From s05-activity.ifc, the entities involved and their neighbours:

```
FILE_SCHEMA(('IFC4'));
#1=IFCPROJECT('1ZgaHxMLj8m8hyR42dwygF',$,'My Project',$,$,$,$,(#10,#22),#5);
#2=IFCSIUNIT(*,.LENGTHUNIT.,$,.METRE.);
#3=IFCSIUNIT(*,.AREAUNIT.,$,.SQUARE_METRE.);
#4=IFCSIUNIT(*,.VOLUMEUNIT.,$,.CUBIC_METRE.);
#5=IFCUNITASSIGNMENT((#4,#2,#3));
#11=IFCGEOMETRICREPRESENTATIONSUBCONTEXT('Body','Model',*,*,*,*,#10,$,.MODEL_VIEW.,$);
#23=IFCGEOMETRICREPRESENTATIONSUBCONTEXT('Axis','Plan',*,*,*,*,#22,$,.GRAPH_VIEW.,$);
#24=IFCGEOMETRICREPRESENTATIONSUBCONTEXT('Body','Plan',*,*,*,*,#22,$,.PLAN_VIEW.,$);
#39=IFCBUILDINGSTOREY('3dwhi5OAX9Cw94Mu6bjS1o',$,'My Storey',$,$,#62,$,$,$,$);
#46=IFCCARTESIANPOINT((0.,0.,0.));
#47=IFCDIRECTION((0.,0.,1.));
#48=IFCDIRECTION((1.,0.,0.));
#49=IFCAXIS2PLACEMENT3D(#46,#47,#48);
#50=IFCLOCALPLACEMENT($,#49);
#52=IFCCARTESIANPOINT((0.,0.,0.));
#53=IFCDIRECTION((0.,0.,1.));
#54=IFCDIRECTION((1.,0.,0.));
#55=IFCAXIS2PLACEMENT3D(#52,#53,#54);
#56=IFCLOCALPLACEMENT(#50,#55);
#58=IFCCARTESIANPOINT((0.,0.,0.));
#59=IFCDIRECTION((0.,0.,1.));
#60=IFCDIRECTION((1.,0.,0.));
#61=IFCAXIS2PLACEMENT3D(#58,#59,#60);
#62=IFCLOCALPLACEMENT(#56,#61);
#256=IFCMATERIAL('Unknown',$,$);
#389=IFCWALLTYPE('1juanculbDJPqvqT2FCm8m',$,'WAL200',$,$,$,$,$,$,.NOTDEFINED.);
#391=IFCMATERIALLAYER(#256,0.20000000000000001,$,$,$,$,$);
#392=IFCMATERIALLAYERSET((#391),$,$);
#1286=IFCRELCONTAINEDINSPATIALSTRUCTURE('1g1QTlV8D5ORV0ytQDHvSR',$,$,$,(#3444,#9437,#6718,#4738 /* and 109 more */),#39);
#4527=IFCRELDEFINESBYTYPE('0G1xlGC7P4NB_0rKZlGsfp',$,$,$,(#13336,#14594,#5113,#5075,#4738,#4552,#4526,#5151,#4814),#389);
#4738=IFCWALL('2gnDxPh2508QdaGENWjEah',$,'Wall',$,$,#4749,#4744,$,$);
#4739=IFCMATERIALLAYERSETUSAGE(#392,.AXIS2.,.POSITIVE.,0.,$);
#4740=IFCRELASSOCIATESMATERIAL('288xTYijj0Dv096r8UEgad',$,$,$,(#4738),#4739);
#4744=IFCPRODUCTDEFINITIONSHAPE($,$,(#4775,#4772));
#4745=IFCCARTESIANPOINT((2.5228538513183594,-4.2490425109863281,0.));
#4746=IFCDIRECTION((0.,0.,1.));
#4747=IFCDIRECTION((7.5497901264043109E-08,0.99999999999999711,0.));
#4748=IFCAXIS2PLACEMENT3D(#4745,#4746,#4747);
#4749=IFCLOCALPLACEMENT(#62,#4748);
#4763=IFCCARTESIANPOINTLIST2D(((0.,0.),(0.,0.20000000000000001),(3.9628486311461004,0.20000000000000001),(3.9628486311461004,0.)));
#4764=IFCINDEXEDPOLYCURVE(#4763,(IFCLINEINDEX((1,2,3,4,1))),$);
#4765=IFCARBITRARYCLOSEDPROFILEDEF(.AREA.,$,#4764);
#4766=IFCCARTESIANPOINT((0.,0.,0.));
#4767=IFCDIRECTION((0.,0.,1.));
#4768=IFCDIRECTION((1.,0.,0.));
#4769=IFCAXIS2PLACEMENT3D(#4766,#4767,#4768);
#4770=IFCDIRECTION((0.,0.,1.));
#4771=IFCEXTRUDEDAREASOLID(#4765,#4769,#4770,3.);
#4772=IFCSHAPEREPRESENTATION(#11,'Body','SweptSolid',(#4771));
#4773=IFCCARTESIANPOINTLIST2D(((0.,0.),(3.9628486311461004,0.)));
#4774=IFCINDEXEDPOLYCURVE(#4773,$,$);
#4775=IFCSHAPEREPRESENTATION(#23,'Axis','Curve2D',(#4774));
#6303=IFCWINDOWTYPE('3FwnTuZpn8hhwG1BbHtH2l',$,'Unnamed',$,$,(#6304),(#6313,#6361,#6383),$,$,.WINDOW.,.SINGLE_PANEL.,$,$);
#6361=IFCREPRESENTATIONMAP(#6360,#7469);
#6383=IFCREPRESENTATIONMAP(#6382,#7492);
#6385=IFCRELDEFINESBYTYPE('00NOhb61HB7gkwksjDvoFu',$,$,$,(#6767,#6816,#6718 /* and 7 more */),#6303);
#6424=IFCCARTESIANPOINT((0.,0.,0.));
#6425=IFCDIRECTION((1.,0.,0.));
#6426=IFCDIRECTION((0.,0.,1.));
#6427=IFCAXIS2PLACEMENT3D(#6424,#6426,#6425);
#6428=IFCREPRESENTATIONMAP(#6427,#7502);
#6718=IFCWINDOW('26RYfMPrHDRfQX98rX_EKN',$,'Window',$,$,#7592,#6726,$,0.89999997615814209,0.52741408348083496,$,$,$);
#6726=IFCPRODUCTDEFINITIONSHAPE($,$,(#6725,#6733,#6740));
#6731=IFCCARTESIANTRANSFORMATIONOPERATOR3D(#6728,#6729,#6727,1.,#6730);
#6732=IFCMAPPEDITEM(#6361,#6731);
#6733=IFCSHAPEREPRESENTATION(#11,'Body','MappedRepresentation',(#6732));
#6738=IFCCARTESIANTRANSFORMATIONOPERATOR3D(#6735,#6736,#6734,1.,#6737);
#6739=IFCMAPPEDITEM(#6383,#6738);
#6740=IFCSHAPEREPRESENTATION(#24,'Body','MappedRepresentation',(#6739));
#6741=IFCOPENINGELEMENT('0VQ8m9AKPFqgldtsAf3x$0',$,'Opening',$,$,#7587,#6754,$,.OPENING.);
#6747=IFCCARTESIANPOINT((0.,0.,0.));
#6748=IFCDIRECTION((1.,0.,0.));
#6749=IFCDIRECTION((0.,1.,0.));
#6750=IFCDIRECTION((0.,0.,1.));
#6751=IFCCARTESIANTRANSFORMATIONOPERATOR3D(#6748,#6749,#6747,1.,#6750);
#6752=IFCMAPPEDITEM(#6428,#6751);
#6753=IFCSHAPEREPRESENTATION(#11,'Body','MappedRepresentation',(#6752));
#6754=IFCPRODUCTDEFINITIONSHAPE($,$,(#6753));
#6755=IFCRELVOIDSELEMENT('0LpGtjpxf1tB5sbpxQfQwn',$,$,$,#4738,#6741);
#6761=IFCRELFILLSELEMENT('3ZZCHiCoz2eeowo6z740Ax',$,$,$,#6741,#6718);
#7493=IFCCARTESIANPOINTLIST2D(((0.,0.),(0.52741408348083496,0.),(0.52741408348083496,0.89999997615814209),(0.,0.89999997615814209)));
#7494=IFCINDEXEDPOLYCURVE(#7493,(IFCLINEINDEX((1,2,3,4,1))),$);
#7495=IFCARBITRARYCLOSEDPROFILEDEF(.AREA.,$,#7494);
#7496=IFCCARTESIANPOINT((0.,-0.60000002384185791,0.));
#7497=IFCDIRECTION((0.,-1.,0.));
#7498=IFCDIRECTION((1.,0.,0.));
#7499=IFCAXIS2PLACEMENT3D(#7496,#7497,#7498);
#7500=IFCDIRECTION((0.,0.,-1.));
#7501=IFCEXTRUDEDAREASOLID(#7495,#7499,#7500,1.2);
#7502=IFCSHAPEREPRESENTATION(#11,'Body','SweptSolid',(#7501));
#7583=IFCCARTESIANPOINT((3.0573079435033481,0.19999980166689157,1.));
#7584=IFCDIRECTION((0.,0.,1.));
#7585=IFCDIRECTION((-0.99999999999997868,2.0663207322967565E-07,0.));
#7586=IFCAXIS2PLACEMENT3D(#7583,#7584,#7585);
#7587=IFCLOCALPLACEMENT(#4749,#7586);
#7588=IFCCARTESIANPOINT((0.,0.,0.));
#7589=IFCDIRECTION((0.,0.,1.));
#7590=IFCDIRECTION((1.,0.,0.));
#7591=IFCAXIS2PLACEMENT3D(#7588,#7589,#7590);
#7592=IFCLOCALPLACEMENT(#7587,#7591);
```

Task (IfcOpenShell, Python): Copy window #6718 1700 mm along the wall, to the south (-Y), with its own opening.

```python
import ifcopenshell
import ifcopenshell.api.feature
import ifcopenshell.api.geometry
import ifcopenshell.api.root
import ifcopenshell.geom
import ifcopenshell.util.element
import ifcopenshell.util.placement
import ifcopenshell.util.shape
import ifcopenshell.util.unit

model = ifcopenshell.open("s05-activity.ifc")
unit_scale = ifcopenshell.util.unit.calculate_unit_scale(model)
settings = ifcopenshell.geom.settings()


def volume(element):
    """Net volume in cubic metres, openings subtracted."""
    shape = ifcopenshell.geom.create_shape(settings, element)
    return ifcopenshell.util.shape.get_volume(shape.geometry)


window = model.by_guid("26RYfMPrHDRfQX98rX_EKN")
opening = window.FillsVoids[0].RelatingOpeningElement
wall = opening.VoidsElements[0].RelatingBuildingElement
before = volume(wall)
shift = ifcopenshell.util.placement.get_local_placement(wall.ObjectPlacement)[:3, 0] * -1.7 / unit_scale

# copy_class copies the void relationship, type, container and properties, but no geometry.
new_opening = ifcopenshell.api.root.copy_class(model, product=opening)
new_opening.Representation = ifcopenshell.util.element.copy_deep(
    model, opening.Representation, exclude=["IfcGeometricRepresentationContext", "IfcRepresentationMap"]
)
new_window = ifcopenshell.api.root.copy_class(model, product=window)
new_window.Representation = ifcopenshell.util.element.copy_deep(
    model, window.Representation, exclude=["IfcGeometricRepresentationContext", "IfcRepresentationMap"]
)
ifcopenshell.api.feature.add_filling(model, opening=new_opening, element=new_window)

for old, new in ((opening, new_opening), (window, new_window)):
    matrix = ifcopenshell.util.placement.get_local_placement(old.ObjectPlacement)
    matrix[:3, 3] += shift
    ifcopenshell.api.geometry.edit_object_placement(model, product=new, matrix=matrix, is_si=False)

after = volume(wall)

print(f"wall volume {before:.3f} -> {after:.3f} m3")

model.write("s05-activity_updated.ifc")
```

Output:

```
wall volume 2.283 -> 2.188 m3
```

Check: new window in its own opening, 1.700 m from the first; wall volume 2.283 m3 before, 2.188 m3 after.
